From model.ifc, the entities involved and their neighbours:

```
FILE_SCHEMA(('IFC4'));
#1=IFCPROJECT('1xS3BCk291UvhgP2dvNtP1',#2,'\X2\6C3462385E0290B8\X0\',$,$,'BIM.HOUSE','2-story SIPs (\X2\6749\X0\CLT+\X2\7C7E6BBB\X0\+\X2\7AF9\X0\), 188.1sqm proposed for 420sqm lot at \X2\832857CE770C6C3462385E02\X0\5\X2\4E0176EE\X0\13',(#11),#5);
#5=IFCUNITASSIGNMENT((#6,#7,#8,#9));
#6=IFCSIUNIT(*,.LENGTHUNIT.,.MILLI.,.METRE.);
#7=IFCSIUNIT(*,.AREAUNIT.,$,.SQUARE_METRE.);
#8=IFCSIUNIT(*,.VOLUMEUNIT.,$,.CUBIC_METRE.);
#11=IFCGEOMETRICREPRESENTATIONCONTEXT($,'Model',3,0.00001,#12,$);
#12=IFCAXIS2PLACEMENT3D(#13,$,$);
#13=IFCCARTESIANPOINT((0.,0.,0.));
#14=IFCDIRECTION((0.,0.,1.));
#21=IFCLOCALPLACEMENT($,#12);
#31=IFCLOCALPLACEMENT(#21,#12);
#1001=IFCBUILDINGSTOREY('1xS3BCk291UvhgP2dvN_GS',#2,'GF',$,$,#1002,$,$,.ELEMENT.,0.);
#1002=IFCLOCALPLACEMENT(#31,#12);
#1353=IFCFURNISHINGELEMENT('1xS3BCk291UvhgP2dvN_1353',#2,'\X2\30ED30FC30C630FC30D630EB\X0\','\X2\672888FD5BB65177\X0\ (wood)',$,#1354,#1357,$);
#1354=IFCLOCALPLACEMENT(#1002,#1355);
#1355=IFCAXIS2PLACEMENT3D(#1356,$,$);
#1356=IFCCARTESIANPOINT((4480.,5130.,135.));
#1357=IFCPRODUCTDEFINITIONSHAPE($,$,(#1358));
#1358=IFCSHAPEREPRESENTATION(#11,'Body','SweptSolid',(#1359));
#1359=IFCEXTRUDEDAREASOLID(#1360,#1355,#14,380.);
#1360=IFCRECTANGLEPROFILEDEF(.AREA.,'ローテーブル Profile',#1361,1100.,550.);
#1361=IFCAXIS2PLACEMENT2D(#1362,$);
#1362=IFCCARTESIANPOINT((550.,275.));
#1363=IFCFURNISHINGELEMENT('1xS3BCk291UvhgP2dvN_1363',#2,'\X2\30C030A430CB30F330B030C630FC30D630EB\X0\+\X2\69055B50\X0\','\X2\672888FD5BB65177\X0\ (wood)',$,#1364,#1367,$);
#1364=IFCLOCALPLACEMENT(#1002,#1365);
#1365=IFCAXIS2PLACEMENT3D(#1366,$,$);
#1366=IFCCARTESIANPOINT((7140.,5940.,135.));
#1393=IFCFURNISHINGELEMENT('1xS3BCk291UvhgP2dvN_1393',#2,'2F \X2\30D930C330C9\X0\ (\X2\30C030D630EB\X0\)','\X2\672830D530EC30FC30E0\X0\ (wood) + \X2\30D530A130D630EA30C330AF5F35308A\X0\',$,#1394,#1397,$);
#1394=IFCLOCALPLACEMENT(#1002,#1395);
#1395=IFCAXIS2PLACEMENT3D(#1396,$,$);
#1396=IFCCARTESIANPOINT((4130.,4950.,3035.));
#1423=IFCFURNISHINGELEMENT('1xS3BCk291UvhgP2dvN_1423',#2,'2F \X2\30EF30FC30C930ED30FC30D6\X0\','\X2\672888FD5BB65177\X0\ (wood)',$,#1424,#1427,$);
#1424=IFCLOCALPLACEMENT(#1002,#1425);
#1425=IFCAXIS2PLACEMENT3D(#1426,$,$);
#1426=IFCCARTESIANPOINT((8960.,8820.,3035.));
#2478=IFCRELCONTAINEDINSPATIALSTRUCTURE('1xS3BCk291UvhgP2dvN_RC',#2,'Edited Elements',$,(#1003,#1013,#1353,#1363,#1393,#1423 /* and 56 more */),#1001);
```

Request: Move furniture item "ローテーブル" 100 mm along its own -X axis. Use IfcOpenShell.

```python
import ifcopenshell
import ifcopenshell.api.geometry
import ifcopenshell.util.placement
import ifcopenshell.util.unit

model = ifcopenshell.open("model.ifc")
unit_scale = ifcopenshell.util.unit.calculate_unit_scale(model)

item = model.by_guid("1xS3BCk291UvhgP2dvN_1353")
matrix = ifcopenshell.util.placement.get_local_placement(item.ObjectPlacement)
matrix[:3, 3] -= matrix[:3, 0] * 0.1 / unit_scale
ifcopenshell.api.geometry.edit_object_placement(model, product=item, matrix=matrix, is_si=False)

print(ifcopenshell.util.placement.get_local_placement(item.ObjectPlacement).round(3) + 0.0)

model.write("model_updated.ifc")
```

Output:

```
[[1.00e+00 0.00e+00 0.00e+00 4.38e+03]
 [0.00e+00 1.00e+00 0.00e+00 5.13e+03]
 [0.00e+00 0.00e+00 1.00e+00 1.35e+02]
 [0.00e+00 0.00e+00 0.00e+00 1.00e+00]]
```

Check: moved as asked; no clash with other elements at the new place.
